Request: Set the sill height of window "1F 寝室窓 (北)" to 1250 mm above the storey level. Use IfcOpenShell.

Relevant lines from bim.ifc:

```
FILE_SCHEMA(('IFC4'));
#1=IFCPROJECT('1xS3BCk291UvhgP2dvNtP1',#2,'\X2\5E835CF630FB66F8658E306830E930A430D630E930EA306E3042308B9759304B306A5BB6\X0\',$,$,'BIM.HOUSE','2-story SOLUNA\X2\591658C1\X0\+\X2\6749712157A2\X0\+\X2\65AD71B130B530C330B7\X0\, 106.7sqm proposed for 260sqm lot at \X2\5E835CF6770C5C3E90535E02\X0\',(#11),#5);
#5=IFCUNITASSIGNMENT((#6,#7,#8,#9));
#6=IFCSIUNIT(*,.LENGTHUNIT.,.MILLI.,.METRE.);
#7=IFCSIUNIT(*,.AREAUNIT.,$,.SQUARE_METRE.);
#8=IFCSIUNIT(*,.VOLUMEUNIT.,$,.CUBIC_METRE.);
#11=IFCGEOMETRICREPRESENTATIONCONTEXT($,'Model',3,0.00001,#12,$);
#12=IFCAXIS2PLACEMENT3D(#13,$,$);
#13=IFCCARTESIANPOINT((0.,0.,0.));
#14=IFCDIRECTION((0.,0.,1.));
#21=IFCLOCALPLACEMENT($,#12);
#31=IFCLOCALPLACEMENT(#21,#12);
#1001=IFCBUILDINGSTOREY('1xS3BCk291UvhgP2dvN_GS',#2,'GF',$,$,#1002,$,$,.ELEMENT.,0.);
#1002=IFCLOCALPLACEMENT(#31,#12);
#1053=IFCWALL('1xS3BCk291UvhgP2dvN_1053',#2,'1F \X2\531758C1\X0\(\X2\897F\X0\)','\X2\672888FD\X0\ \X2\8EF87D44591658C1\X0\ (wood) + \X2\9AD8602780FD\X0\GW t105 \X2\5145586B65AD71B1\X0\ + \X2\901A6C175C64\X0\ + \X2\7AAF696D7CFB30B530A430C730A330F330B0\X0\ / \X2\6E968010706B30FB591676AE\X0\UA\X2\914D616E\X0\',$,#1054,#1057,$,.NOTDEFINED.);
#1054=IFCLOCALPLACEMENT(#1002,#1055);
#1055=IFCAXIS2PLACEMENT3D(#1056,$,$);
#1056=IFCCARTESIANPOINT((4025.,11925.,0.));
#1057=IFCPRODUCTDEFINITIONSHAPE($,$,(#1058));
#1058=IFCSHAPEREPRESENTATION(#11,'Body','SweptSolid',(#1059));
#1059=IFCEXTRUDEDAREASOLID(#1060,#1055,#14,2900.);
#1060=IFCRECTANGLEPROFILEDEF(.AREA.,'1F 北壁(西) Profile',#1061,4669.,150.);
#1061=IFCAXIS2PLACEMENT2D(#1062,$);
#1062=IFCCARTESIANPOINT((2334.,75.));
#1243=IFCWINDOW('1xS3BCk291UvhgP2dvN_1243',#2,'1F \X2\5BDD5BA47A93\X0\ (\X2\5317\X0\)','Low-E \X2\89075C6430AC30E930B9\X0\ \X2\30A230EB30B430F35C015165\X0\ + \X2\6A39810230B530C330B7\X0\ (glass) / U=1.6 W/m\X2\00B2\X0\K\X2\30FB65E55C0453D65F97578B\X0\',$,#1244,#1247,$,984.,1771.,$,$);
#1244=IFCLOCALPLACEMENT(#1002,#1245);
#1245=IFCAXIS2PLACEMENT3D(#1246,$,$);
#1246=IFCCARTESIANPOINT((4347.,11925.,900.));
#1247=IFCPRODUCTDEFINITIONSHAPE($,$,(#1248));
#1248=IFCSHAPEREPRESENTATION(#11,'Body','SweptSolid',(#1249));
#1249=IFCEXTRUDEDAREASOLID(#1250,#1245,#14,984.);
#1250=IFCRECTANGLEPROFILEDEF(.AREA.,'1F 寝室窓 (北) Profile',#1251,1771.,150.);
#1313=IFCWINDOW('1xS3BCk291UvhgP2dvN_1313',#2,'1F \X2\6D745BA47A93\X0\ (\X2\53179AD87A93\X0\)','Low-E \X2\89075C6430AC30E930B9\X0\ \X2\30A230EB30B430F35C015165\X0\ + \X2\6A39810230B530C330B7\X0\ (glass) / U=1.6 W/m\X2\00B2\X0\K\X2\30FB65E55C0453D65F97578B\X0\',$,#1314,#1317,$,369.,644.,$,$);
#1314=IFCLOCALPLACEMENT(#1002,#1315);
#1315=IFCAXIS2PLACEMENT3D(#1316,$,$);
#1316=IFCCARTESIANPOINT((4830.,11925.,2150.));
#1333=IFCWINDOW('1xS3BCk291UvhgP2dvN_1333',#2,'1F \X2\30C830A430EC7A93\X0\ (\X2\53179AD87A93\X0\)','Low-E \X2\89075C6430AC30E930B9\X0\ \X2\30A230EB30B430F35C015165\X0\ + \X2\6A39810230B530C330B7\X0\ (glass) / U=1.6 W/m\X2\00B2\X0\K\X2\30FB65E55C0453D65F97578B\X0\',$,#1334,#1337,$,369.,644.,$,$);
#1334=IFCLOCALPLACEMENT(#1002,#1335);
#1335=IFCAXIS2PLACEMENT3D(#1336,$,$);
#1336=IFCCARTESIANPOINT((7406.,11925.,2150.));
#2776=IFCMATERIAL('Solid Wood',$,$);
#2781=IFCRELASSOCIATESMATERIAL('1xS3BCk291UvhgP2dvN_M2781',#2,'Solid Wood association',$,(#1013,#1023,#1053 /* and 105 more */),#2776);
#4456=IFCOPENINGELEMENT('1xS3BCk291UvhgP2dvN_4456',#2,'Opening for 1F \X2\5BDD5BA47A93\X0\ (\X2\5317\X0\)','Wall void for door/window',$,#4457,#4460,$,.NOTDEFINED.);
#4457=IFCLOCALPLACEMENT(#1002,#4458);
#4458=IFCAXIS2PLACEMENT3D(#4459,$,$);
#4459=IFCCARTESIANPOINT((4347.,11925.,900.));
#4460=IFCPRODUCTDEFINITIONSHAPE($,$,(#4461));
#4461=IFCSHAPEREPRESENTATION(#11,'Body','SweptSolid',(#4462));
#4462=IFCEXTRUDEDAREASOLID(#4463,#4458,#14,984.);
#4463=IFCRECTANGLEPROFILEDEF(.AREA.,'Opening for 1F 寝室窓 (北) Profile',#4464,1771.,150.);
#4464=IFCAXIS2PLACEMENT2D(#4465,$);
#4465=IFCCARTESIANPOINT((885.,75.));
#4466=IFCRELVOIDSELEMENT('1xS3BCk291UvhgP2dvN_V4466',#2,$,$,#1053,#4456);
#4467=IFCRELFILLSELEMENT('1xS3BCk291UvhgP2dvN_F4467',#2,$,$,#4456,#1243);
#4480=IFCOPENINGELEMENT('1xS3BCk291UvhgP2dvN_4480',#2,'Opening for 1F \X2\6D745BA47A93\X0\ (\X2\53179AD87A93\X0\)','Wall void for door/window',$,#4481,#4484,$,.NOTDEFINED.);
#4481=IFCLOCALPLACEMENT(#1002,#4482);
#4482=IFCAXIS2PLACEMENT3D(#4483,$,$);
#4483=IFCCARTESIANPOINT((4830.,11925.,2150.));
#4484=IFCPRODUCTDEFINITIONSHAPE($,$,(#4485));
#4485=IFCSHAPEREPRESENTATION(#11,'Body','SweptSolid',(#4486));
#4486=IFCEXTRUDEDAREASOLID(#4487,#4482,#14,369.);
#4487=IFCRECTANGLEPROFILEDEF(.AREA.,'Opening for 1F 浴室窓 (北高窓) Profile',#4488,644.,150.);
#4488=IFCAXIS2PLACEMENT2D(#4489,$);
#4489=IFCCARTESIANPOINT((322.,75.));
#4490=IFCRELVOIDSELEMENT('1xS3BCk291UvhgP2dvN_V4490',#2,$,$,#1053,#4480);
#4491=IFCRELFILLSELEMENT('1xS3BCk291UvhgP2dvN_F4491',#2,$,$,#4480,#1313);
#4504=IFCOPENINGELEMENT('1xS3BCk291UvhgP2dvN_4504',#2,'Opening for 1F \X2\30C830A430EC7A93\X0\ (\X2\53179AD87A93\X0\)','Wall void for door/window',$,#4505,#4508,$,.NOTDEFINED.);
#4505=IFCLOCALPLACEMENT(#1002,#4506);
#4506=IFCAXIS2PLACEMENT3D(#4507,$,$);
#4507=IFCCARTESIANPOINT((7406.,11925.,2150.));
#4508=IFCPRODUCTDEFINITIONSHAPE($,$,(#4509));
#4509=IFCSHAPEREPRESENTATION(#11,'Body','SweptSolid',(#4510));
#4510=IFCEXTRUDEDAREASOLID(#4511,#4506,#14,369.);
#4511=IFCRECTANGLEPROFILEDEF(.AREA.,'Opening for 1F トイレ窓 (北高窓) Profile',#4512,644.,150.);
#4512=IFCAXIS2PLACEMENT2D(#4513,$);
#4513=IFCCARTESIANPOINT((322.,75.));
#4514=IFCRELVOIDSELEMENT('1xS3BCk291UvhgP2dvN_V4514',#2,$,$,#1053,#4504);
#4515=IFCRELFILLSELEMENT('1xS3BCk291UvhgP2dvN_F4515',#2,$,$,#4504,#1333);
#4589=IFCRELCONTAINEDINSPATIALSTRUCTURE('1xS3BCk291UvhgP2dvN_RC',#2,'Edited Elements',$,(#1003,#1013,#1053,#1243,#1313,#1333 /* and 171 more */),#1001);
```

```python
import numpy as np
import ifcopenshell
import ifcopenshell.api.geometry
import ifcopenshell.geom
import ifcopenshell.util.element
import ifcopenshell.util.placement
import ifcopenshell.util.shape
import ifcopenshell.util.unit

model = ifcopenshell.open("bim.ifc")
unit_scale = ifcopenshell.util.unit.calculate_unit_scale(model)

window = model.by_guid("1xS3BCk291UvhgP2dvN_1243")
opening = window.FillsVoids[0].RelatingOpeningElement
storey = ifcopenshell.util.element.get_container(window, ifc_class="IfcBuildingStorey")
level = ifcopenshell.util.placement.get_local_placement(storey.ObjectPlacement)[2, 3]

# The opening's origin need not be at the sill, so measure its lowest point.
shape = ifcopenshell.geom.create_shape(ifcopenshell.geom.settings(), opening)
bottom = ifcopenshell.util.shape.get_shape_bottom_elevation(shape, shape.geometry) / unit_scale
dz = level + 1250.0 - bottom

shift = np.array([0.0, 0.0, dz])
# The window is not placed relative to its opening, so move both.
for product in (opening, window):
    matrix = ifcopenshell.util.placement.get_local_placement(product.ObjectPlacement)
    matrix[:3, 3] += shift
    ifcopenshell.api.geometry.edit_object_placement(model, product=product, matrix=matrix, is_si=False)

print(f"moved by {dz * unit_scale:+.3f} m")

model.write("bim_edited.ifc")
```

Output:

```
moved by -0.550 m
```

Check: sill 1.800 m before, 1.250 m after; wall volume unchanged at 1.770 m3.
